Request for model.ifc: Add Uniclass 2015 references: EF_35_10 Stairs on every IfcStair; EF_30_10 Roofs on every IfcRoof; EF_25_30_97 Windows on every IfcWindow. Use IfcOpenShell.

First a look at what the model holds.

```python
import ifcopenshell

model = ifcopenshell.open("model.ifc")
print(model.schema)
print("classifications:", [c.Name for c in model.by_type("IfcClassification")])
for ifc_class in ("IfcDoor", "IfcRoof", "IfcStair", "IfcWall", "IfcWindow"):
    print(ifc_class, len(model.by_type(ifc_class)))
```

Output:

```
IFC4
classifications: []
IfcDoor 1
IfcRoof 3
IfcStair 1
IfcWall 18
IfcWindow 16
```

```python
import ifcopenshell
import ifcopenshell.api.classification

model = ifcopenshell.open("model.ifc")

system = ifcopenshell.api.classification.add_classification(model, classification="Uniclass 2015")

codes = {
    "IfcStair": ("EF_35_10", "Stairs"),
    "IfcRoof": ("EF_30_10", "Roofs"),
    "IfcWindow": ("EF_25_30_97", "Windows"),
}
for ifc_class, (code, name) in codes.items():
    products = model.by_type(ifc_class)
    ifcopenshell.api.classification.add_reference(
        model, products=products, classification=system, identification=code, name=name
    )
    print(code, len(products))

model.write("model_updated.ifc")
```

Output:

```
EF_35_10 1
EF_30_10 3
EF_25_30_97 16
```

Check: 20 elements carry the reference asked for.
